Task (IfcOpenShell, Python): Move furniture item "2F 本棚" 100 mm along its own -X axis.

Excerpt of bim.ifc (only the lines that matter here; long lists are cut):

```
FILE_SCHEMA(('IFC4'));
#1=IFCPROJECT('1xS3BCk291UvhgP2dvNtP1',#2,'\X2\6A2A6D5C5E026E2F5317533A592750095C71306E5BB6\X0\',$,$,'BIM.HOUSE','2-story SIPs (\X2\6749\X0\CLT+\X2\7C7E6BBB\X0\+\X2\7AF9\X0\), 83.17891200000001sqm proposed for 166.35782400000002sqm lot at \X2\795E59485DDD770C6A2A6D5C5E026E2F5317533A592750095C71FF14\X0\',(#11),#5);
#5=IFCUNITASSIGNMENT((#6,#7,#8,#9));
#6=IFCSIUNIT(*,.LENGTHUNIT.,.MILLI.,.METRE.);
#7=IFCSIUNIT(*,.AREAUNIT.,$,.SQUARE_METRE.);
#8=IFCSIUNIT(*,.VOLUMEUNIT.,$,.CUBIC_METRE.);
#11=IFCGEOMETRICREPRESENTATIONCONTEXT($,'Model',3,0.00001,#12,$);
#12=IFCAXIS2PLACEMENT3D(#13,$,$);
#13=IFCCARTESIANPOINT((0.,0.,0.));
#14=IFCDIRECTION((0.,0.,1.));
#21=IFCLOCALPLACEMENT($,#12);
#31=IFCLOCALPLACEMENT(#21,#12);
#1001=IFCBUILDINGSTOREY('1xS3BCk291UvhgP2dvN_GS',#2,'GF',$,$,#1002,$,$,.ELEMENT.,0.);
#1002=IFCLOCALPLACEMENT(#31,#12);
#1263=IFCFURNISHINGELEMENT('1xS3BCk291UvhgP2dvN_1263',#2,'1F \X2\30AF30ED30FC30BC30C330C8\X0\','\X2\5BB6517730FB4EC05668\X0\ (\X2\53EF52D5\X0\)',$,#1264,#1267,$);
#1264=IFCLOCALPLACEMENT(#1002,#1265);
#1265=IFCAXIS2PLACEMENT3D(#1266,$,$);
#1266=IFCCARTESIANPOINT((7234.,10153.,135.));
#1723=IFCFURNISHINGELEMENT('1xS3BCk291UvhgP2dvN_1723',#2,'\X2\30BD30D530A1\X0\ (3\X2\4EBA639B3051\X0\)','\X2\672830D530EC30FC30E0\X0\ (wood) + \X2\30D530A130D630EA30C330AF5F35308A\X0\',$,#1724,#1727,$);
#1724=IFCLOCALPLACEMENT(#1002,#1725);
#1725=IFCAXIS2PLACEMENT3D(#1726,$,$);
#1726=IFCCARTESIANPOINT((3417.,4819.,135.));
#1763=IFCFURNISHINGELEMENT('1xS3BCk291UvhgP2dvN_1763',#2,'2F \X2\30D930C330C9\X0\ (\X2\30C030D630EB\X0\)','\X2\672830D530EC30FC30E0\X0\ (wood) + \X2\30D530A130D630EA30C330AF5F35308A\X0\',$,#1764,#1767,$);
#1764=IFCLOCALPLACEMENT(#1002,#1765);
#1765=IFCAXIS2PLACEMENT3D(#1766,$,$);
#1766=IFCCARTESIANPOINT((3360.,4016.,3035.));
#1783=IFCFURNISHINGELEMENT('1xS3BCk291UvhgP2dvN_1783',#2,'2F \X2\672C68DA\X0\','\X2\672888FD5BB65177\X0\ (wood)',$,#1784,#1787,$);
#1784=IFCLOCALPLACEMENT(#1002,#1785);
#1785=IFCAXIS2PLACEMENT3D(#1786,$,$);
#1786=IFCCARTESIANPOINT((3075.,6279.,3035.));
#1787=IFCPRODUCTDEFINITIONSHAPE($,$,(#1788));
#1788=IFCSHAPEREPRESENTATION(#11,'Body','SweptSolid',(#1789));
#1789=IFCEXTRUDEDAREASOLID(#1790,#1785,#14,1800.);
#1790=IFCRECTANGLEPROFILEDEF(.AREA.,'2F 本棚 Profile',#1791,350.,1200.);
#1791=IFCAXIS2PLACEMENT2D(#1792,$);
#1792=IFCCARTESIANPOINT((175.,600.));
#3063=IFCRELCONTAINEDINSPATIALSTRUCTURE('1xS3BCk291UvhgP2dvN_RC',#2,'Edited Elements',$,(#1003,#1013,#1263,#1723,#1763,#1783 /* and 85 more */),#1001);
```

```python
import ifcopenshell
import ifcopenshell.api.geometry
import ifcopenshell.util.placement

model = ifcopenshell.open("bim.ifc")

item = model.by_id(1783)
matrix = ifcopenshell.util.placement.get_local_placement(item.ObjectPlacement)
matrix[:3, 3] -= matrix[:3, 0] * 100.0
ifcopenshell.api.geometry.edit_object_placement(model, product=item, matrix=matrix, is_si=False)

print(ifcopenshell.util.placement.get_local_placement(item.ObjectPlacement).round(3) + 0.0)

model.write("bim_updated.ifc")
```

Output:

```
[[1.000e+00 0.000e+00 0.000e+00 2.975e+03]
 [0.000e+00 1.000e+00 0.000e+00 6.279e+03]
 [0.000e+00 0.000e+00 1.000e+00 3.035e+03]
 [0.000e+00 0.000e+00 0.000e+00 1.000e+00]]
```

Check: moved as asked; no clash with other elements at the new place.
